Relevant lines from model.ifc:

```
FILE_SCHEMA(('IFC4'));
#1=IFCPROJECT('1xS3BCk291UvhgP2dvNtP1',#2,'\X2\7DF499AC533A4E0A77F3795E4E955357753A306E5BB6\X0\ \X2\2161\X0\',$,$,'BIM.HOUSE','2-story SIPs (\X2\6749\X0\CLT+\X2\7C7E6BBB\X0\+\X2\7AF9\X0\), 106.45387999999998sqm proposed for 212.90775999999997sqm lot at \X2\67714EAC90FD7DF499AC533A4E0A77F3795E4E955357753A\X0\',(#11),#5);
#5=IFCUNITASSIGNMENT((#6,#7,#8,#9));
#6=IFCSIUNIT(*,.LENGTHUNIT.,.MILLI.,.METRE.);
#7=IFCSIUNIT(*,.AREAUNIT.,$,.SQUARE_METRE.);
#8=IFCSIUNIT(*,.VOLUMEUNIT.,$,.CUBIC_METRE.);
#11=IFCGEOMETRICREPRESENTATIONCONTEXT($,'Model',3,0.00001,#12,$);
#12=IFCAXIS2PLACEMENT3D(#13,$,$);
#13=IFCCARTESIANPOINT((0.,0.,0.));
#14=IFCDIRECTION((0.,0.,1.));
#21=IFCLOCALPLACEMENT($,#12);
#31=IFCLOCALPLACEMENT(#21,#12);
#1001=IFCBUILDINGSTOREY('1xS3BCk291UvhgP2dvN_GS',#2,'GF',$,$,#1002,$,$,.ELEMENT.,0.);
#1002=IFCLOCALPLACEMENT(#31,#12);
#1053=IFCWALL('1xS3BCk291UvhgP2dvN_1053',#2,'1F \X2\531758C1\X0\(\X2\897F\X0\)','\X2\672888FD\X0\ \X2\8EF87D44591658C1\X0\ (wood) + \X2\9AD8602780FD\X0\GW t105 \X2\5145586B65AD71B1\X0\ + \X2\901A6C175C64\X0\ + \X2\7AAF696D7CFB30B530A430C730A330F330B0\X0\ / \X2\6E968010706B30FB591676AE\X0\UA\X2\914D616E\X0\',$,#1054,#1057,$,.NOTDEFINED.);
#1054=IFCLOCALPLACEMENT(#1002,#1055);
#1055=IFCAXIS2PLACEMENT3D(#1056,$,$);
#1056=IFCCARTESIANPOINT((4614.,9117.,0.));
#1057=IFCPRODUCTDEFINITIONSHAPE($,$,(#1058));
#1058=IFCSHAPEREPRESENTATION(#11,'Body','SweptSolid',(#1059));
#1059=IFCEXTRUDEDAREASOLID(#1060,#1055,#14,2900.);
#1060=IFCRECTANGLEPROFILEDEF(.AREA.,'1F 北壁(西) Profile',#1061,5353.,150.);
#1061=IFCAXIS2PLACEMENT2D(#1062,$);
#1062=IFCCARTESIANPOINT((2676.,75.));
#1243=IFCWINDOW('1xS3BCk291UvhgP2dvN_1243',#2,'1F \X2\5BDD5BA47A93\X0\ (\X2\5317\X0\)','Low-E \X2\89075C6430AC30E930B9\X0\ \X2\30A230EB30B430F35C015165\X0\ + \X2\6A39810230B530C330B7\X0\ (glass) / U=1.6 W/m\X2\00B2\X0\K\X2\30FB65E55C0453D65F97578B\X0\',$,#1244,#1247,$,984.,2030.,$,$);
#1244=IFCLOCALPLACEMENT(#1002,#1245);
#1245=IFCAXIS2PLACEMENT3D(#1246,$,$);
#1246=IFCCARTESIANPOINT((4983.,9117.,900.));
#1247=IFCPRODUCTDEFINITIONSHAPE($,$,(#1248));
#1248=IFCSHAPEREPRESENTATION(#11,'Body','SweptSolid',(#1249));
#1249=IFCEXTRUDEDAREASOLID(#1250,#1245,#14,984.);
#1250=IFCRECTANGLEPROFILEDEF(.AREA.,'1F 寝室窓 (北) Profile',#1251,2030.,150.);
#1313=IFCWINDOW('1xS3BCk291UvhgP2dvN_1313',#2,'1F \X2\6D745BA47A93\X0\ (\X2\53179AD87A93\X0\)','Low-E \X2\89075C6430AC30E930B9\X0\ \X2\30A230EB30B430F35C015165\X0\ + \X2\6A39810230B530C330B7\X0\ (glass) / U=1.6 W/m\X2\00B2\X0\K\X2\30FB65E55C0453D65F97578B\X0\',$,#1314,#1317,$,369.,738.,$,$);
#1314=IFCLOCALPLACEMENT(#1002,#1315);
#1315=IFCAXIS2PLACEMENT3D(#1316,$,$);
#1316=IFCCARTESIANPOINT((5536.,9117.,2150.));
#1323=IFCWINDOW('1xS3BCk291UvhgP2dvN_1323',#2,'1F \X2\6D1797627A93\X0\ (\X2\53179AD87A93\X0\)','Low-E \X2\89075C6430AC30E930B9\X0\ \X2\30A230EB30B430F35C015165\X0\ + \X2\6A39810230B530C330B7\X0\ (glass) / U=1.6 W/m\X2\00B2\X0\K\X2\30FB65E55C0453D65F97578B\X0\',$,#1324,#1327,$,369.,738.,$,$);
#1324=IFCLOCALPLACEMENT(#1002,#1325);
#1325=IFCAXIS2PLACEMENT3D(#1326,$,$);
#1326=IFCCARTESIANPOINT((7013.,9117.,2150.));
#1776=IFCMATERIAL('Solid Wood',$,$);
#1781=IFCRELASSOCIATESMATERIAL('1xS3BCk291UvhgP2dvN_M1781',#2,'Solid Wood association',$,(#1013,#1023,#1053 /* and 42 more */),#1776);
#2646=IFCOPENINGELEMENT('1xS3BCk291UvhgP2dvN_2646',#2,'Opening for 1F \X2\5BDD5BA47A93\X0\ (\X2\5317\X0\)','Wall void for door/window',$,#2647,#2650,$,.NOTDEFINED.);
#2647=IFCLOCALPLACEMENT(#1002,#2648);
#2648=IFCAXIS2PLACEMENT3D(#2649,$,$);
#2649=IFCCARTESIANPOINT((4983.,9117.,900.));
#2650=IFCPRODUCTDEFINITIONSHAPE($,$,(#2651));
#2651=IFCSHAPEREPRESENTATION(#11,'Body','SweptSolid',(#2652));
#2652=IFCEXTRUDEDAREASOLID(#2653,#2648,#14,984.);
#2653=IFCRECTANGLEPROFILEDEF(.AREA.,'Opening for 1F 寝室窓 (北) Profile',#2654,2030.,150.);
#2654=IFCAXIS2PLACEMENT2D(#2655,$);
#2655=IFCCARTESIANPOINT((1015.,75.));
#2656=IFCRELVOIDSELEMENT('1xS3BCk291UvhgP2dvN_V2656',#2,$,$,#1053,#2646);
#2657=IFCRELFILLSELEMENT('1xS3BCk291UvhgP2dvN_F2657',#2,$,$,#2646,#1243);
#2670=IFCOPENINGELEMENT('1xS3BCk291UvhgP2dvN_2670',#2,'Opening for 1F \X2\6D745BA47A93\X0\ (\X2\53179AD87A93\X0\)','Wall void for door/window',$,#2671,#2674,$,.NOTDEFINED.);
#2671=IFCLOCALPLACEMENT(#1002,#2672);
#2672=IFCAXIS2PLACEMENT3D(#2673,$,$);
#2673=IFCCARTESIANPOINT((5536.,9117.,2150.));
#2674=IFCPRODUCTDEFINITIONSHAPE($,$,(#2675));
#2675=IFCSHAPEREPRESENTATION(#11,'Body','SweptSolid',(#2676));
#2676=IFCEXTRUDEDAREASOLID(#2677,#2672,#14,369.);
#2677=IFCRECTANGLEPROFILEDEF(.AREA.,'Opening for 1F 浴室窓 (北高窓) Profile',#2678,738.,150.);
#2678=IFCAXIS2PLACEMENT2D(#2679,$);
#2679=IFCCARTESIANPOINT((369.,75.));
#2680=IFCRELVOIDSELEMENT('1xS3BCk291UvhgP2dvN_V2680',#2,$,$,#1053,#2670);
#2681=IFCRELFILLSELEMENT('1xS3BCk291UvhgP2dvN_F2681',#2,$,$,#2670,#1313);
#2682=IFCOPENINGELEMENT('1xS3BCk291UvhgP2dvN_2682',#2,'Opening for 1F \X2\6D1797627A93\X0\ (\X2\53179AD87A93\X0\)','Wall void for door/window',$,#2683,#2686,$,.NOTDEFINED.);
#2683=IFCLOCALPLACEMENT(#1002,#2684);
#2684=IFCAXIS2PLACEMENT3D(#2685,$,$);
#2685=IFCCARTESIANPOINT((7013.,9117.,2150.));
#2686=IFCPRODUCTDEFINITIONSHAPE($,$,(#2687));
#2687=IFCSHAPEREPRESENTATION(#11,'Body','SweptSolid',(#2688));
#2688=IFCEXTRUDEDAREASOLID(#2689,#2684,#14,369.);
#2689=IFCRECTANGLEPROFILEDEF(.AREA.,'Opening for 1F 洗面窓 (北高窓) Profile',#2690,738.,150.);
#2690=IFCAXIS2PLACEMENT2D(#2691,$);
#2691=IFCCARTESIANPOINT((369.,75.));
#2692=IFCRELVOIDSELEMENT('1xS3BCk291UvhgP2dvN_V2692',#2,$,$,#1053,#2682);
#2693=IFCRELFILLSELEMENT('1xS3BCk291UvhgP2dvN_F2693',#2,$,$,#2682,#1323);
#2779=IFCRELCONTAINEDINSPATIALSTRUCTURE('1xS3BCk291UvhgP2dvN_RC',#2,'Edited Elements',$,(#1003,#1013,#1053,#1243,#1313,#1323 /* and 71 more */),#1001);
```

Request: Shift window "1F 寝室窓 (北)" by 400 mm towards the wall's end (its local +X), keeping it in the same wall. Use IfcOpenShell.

```python
import ifcopenshell
import ifcopenshell.api.geometry
import ifcopenshell.util.placement

model = ifcopenshell.open("model.ifc")

window = model.by_guid("1xS3BCk291UvhgP2dvN_1243")
opening = window.FillsVoids[0].RelatingOpeningElement
wall = opening.VoidsElements[0].RelatingBuildingElement

wall_matrix = ifcopenshell.util.placement.get_local_placement(wall.ObjectPlacement)
shift = wall_matrix[:3, 0] * 400.0
before = ifcopenshell.util.placement.get_local_placement(window.ObjectPlacement)[:3, 3].copy()

# The window is not placed relative to its opening, so move both.
for product in (opening, window):
    matrix = ifcopenshell.util.placement.get_local_placement(product.ObjectPlacement)
    matrix[:3, 3] += shift
    ifcopenshell.api.geometry.edit_object_placement(model, product=product, matrix=matrix, is_si=False)

after = ifcopenshell.util.placement.get_local_placement(window.ObjectPlacement)[:3, 3]
print("window moved by", (after - before).round(3) + 0.0)

model.write("model_updated.ifc")
```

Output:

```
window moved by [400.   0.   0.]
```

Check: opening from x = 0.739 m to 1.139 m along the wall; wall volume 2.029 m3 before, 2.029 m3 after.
